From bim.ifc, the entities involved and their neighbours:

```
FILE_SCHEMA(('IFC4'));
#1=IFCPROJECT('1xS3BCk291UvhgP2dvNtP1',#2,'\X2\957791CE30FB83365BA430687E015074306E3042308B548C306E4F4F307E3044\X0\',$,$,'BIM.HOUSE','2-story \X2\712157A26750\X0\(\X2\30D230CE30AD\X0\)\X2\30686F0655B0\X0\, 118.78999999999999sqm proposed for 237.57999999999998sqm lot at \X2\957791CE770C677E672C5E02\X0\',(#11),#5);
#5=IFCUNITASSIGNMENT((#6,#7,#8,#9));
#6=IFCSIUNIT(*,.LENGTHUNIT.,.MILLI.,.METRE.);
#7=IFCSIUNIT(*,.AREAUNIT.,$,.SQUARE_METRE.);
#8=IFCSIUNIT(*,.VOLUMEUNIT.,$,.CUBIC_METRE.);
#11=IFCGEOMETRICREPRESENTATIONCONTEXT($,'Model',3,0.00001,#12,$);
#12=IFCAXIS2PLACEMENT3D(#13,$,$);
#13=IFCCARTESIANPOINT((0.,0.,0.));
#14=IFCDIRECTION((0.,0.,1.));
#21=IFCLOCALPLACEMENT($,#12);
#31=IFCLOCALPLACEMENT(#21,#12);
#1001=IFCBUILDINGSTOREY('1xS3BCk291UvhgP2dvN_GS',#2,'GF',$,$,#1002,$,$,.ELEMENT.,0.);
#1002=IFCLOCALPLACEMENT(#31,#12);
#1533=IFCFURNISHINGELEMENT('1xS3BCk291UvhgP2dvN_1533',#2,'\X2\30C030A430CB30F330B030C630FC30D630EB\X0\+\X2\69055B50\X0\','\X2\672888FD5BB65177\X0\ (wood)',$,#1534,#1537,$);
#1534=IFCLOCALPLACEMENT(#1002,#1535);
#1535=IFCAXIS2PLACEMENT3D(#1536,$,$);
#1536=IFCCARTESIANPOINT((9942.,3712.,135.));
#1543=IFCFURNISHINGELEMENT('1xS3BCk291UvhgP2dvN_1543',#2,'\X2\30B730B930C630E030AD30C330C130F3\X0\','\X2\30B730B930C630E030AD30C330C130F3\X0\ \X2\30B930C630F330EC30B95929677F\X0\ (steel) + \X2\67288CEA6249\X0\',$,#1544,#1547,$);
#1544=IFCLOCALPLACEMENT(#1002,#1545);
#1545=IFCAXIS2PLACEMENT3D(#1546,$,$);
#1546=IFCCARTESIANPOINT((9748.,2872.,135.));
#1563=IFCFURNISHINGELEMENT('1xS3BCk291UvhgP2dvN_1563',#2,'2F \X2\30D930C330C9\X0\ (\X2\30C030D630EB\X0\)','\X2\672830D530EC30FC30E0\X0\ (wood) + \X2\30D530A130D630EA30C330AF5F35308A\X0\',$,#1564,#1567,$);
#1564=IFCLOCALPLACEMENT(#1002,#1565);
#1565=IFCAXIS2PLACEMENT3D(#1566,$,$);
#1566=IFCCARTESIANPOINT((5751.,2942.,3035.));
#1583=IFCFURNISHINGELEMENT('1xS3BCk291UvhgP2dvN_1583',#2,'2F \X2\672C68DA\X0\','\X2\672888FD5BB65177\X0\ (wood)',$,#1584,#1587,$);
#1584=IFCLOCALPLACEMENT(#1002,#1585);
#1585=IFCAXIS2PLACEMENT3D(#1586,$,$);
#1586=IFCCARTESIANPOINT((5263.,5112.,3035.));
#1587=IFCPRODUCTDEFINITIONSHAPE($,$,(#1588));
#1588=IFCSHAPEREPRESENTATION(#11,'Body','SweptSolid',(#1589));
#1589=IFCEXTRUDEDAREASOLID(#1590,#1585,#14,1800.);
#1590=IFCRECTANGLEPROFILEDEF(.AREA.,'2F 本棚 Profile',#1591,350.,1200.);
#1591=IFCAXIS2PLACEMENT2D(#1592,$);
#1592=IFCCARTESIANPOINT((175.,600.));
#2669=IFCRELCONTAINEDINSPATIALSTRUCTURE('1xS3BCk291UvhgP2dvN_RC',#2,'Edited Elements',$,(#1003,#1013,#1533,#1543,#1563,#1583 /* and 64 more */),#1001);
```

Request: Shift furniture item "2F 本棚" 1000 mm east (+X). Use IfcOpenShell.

```python
import ifcopenshell
import ifcopenshell.api.geometry
import ifcopenshell.util.placement
import ifcopenshell.util.unit

model = ifcopenshell.open("bim.ifc")
unit_scale = ifcopenshell.util.unit.calculate_unit_scale(model)

item = model.by_guid("1xS3BCk291UvhgP2dvN_1583")
matrix = ifcopenshell.util.placement.get_local_placement(item.ObjectPlacement)
matrix[0, 3] += 1 / unit_scale
ifcopenshell.api.geometry.edit_object_placement(model, product=item, matrix=matrix, is_si=False)

print(ifcopenshell.util.placement.get_local_placement(item.ObjectPlacement).round(3) + 0.0)

model.write("bim_updated.ifc")
```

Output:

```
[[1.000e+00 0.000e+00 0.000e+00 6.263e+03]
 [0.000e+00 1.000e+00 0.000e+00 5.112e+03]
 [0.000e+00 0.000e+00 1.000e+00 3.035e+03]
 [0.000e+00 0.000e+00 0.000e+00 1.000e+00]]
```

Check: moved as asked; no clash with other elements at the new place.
